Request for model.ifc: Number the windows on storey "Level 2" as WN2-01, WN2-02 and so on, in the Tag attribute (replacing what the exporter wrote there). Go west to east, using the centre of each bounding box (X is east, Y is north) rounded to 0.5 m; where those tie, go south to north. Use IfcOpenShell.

First a look at what the model holds.

```python
import ifcopenshell
import ifcopenshell.util.element
import ifcopenshell.util.placement

model = ifcopenshell.open("model.ifc")
print(model.schema)
storey = next(s for s in model.by_type("IfcBuildingStorey") if s.Name == "Level 2")
windows = [e for e in ifcopenshell.util.element.get_decomposition(storey) if e.is_a("IfcWindow")]
for e in sorted(windows, key=lambda e: e.id()):
    origin = ifcopenshell.util.placement.get_local_placement(e.ObjectPlacement)[:3, 3]
    print(e.id(), e.Tag, e.Name, origin.round(2) + 0.0, sep=" | ")
```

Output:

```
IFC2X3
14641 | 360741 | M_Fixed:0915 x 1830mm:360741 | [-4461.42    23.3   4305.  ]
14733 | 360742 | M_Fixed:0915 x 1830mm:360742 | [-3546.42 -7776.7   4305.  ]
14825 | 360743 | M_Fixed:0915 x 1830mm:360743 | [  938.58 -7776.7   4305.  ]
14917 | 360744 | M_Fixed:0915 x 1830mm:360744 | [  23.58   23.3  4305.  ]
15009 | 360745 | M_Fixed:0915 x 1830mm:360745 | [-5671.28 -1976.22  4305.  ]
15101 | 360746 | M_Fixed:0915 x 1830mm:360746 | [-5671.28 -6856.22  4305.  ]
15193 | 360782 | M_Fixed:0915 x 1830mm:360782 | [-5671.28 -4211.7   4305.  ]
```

```python
import ifcopenshell
import ifcopenshell.geom
import ifcopenshell.util.element
import ifcopenshell.util.shape

model = ifcopenshell.open("model.ifc")
settings = ifcopenshell.geom.settings()
settings.set("use-world-coords", True)


def centre(element):
    shape = ifcopenshell.geom.create_shape(settings, element)
    return ifcopenshell.util.shape.get_bbox_centroid(shape.geometry)


storey = next(s for s in model.by_type("IfcBuildingStorey") if s.Name == "Level 2")
windows = [e for e in ifcopenshell.util.element.get_decomposition(storey) if e.is_a("IfcWindow")]

# Insertion points can sit at a corner or the storey origin, so sort by the geometry (in metres).
centres = {e: centre(e) for e in windows}
windows.sort(key=lambda e: (round(centres[e][0] / 0.5), centres[e][1]))

for i, e in enumerate(windows, start=1):
    number = f"WN2-{i:02d}"
    e.Tag = number
    print(e.id(), number)

model.write("model_v2.ifc")
```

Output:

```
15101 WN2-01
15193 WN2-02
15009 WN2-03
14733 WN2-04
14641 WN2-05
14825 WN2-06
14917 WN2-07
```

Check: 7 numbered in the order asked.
